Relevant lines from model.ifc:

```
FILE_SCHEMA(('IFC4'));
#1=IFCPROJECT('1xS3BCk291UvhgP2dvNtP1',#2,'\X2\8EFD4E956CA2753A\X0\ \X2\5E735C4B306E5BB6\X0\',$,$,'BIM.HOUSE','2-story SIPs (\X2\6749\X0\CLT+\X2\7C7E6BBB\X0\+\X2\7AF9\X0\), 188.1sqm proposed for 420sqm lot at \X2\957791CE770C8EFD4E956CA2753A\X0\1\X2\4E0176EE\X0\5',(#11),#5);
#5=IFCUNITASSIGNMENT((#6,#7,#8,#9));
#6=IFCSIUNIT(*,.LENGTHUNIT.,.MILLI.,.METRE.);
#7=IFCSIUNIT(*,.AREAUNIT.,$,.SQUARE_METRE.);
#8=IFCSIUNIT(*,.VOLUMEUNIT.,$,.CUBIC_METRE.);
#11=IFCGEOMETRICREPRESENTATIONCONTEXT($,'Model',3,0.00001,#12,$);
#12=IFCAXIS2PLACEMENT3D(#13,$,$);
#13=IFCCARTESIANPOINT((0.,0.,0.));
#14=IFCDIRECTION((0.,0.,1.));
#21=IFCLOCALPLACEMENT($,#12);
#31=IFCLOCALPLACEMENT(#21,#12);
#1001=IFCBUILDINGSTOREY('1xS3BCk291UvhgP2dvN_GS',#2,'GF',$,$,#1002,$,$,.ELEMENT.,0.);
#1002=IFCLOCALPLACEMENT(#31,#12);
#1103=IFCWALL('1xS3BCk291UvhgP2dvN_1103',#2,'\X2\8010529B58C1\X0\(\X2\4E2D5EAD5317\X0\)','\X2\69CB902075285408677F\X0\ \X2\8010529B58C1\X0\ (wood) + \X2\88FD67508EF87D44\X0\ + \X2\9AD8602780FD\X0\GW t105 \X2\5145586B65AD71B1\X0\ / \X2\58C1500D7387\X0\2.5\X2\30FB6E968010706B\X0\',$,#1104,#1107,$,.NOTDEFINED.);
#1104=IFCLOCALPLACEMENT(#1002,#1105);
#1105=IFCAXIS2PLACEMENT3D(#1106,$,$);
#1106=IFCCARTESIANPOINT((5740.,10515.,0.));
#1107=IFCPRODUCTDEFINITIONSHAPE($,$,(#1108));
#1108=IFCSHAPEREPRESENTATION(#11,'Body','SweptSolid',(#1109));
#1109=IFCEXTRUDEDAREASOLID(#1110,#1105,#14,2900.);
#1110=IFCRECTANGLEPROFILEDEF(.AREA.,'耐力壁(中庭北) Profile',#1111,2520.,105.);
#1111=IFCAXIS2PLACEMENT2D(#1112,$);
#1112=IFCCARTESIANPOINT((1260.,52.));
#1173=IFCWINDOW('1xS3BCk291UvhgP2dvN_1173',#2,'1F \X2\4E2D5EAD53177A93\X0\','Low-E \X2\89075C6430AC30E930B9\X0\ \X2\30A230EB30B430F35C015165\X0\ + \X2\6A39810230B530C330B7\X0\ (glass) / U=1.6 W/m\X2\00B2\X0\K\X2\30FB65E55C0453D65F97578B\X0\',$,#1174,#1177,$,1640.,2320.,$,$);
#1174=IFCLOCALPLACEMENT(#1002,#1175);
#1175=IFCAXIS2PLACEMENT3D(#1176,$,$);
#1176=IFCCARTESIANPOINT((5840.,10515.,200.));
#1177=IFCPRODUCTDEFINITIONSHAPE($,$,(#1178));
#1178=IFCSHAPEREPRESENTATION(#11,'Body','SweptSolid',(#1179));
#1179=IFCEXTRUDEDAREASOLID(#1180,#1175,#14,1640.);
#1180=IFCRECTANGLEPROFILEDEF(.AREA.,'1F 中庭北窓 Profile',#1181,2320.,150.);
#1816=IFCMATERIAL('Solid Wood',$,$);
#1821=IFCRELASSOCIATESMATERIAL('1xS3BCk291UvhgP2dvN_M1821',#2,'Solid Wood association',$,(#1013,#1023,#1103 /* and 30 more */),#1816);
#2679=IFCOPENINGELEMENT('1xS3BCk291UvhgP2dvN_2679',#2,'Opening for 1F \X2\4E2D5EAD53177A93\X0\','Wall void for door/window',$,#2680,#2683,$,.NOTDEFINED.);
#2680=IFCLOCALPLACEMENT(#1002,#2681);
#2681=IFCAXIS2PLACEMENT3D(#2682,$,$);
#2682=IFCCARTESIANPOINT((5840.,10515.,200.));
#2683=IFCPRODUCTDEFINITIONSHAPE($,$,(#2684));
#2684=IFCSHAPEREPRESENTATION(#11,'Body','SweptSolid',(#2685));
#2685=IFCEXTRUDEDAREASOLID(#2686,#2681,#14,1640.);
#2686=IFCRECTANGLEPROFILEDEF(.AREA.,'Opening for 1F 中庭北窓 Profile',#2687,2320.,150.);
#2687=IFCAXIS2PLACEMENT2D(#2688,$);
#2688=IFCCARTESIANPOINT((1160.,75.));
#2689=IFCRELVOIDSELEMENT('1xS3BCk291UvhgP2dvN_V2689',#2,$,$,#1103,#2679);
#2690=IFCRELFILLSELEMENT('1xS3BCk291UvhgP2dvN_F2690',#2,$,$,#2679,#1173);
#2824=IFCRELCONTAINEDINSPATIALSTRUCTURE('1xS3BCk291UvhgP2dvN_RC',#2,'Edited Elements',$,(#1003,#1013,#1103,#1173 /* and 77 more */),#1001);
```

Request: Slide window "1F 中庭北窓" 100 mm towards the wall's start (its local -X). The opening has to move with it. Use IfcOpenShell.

```python
import ifcopenshell
import ifcopenshell.api.geometry
import ifcopenshell.util.placement

model = ifcopenshell.open("model.ifc")

window = model.by_guid("1xS3BCk291UvhgP2dvN_1173")
opening = window.FillsVoids[0].RelatingOpeningElement
wall = opening.VoidsElements[0].RelatingBuildingElement

wall_matrix = ifcopenshell.util.placement.get_local_placement(wall.ObjectPlacement)
shift = wall_matrix[:3, 0] * -100.0
before = ifcopenshell.util.placement.get_local_placement(window.ObjectPlacement)[:3, 3].copy()

# The window is not placed relative to its opening, so move both.
for product in (opening, window):
    matrix = ifcopenshell.util.placement.get_local_placement(product.ObjectPlacement)
    matrix[:3, 3] += shift
    ifcopenshell.api.geometry.edit_object_placement(model, product=product, matrix=matrix, is_si=False)

after = ifcopenshell.util.placement.get_local_placement(window.ObjectPlacement)[:3, 3]
print("window moved by", (after - before).round(3) + 0.0)

model.write("model-out.ifc")
```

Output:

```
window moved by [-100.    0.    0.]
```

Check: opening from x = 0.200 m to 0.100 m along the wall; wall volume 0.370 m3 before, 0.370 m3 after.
